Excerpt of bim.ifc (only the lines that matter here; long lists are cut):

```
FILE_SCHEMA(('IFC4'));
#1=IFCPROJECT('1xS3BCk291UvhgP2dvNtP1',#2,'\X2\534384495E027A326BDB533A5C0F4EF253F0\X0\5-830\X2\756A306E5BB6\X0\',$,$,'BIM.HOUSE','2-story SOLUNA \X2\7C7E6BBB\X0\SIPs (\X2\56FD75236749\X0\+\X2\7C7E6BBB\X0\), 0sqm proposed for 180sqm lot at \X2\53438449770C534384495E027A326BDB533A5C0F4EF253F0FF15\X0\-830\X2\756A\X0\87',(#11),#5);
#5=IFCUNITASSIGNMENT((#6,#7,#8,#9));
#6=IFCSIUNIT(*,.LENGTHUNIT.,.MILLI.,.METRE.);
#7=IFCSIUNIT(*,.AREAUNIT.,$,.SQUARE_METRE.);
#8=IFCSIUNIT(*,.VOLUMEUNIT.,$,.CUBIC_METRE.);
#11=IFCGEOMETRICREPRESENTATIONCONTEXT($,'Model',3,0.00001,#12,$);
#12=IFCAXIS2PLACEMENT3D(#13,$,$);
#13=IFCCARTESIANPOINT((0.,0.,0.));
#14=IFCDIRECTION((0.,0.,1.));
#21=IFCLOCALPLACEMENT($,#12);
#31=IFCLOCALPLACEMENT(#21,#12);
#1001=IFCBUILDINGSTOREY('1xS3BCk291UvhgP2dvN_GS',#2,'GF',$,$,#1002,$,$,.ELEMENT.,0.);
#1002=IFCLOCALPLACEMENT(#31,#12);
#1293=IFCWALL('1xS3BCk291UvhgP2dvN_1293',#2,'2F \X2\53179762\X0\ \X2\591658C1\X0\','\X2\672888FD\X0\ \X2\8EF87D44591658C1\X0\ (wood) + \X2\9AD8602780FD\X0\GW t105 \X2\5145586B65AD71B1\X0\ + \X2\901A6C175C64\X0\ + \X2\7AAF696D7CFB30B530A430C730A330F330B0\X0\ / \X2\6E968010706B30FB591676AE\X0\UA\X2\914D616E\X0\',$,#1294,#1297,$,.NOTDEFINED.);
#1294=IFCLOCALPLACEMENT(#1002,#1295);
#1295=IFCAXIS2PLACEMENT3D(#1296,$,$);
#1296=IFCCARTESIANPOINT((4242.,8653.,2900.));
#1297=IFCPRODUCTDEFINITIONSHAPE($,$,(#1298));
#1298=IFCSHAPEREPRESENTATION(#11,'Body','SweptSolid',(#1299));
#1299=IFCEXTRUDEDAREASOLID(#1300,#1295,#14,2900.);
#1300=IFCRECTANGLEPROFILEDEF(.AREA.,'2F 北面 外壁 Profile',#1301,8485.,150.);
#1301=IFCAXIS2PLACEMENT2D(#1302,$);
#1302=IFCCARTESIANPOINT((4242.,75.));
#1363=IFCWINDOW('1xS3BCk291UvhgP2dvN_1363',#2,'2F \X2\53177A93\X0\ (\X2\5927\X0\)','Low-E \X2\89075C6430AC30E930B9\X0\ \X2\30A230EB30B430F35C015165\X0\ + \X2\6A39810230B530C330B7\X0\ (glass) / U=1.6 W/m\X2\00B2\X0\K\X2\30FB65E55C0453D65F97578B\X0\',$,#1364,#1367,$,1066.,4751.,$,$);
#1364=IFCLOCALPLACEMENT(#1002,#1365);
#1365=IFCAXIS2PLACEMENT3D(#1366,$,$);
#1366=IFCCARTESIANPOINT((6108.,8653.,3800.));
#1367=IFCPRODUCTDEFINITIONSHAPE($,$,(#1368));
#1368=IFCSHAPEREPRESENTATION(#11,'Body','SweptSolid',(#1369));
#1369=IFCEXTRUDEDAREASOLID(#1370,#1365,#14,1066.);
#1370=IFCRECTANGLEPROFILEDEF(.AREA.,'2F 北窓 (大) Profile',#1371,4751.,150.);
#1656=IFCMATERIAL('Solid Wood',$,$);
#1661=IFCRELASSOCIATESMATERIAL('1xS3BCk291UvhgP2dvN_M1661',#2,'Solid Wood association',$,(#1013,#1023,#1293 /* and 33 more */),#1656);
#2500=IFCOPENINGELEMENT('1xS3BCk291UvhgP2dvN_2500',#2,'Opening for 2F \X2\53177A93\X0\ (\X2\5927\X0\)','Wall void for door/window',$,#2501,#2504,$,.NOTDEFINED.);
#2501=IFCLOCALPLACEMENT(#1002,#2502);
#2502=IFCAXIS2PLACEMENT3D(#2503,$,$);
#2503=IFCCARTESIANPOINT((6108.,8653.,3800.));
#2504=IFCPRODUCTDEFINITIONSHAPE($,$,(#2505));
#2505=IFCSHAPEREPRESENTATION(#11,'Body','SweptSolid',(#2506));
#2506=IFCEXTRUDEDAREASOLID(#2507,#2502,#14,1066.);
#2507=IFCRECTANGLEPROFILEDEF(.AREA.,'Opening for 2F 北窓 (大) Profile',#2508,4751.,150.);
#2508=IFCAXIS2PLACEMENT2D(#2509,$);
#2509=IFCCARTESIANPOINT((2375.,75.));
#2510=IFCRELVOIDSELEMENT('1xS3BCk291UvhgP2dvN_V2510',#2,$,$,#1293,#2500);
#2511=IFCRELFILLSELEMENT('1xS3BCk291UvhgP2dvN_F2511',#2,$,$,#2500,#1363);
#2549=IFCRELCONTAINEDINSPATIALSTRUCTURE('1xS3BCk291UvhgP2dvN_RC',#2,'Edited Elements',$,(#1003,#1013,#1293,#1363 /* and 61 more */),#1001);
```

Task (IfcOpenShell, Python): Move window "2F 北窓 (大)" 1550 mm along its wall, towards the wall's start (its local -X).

```python
import ifcopenshell
import ifcopenshell.api.geometry
import ifcopenshell.util.placement
import ifcopenshell.util.unit

model = ifcopenshell.open("bim.ifc")
unit_scale = ifcopenshell.util.unit.calculate_unit_scale(model)

window = model.by_guid("1xS3BCk291UvhgP2dvN_1363")
opening = window.FillsVoids[0].RelatingOpeningElement
wall = opening.VoidsElements[0].RelatingBuildingElement

wall_matrix = ifcopenshell.util.placement.get_local_placement(wall.ObjectPlacement)
shift = wall_matrix[:3, 0] * -1.55 / unit_scale
before = ifcopenshell.util.placement.get_local_placement(window.ObjectPlacement)[:3, 3].copy()

# The window is not placed relative to its opening, so move both.
for product in (opening, window):
    matrix = ifcopenshell.util.placement.get_local_placement(product.ObjectPlacement)
    matrix[:3, 3] += shift
    ifcopenshell.api.geometry.edit_object_placement(model, product=product, matrix=matrix, is_si=False)

after = ifcopenshell.util.placement.get_local_placement(window.ObjectPlacement)[:3, 3]
print("window moved by", (after - before).round(3) + 0.0)

model.write("bim_rev.ifc")
```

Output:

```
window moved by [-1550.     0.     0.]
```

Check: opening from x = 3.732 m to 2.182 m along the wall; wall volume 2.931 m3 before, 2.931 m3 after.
